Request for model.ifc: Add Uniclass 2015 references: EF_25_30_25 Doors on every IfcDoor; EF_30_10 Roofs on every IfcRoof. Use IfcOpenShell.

First a look at what the model holds.

```python
import ifcopenshell

model = ifcopenshell.open("model.ifc")
print(model.schema)
print("classifications:", [c.Name for c in model.by_type("IfcClassification")])
for ifc_class in ("IfcDoor", "IfcRoof", "IfcStair", "IfcWall", "IfcWindow"):
    print(ifc_class, len(model.by_type(ifc_class)))
```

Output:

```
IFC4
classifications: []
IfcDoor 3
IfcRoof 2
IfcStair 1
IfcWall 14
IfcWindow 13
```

```python
import ifcopenshell
import ifcopenshell.api.classification

model = ifcopenshell.open("model.ifc")

system = ifcopenshell.api.classification.add_classification(model, classification="Uniclass 2015")

codes = {
    "IfcDoor": ("EF_25_30_25", "Doors"),
    "IfcRoof": ("EF_30_10", "Roofs"),
}
for ifc_class, (code, name) in codes.items():
    products = model.by_type(ifc_class)
    ifcopenshell.api.classification.add_reference(
        model, products=products, classification=system, identification=code, name=name
    )
    print(code, len(products))

model.write("model_rev.ifc")
```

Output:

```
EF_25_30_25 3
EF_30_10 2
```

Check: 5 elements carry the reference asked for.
